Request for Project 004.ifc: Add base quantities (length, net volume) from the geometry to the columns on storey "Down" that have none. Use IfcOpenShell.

First a look at what the model holds.

```python
import ifcopenshell
import ifcopenshell.util.element
import ifcopenshell.util.unit

model = ifcopenshell.open("Project 004.ifc")
print(model.schema)
for unit_type in ("LENGTHUNIT", "AREAUNIT", "VOLUMEUNIT"):
    print(unit_type, ifcopenshell.util.unit.calculate_unit_scale(model, unit_type))
storey = next(s for s in model.by_type("IfcBuildingStorey") if s.Name == "Down")
columns = [e for e in ifcopenshell.util.element.get_decomposition(storey) if e.is_a("IfcColumn")]
for e in sorted(columns, key=lambda e: e.id()):
    print(e.id(), e.is_a(), e.Name, list(ifcopenshell.util.element.get_psets(e, qtos_only=True)), sep=" | ")
```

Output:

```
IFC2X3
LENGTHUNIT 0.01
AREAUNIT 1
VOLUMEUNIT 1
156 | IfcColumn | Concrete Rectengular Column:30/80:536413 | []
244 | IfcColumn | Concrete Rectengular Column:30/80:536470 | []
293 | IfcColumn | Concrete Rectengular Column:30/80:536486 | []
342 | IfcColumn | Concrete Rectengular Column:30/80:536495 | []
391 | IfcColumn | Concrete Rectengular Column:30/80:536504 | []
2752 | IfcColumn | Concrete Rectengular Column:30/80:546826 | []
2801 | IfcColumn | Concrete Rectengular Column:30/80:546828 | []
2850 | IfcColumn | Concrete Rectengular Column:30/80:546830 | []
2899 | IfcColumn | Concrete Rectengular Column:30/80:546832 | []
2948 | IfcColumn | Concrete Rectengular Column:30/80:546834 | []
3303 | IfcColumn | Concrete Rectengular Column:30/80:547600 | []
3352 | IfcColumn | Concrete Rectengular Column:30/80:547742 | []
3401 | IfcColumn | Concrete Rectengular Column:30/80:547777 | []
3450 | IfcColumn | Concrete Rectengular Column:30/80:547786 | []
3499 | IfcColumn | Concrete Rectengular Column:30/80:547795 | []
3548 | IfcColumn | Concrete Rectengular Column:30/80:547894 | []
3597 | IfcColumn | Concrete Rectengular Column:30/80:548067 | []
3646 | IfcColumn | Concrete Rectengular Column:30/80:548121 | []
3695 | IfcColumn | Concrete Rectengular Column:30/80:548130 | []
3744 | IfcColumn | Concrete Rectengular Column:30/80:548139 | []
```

```python
import ifcopenshell
import ifcopenshell.api.pset
import ifcopenshell.geom
import ifcopenshell.util.element
import ifcopenshell.util.shape
import ifcopenshell.util.unit

model = ifcopenshell.open("Project 004.ifc")
unit_scale = ifcopenshell.util.unit.calculate_unit_scale(model)
volume_scale = ifcopenshell.util.unit.calculate_unit_scale(model, "VOLUMEUNIT")
settings = ifcopenshell.geom.settings()

storey = next(s for s in model.by_type("IfcBuildingStorey") if s.Name == "Down")
columns = [e for e in ifcopenshell.util.element.get_decomposition(storey) if e.is_a("IfcColumn")]

for e in sorted(columns, key=lambda e: e.id()):
    if ifcopenshell.util.element.get_psets(e, qtos_only=True, should_inherit=False):
        continue
    # Geometry comes back in metres, in the element's own axes.
    shape = ifcopenshell.geom.create_shape(settings, e)
    values = {
        "Length": ifcopenshell.util.shape.get_z(shape.geometry) / unit_scale,
        "NetVolume": ifcopenshell.util.shape.get_volume(shape.geometry) / volume_scale,
    }
    qto = ifcopenshell.api.pset.add_qto(model, product=e, name="BaseQuantities")
    ifcopenshell.api.pset.edit_qto(model, qto=qto, properties=values)
    print(e.id(), {k: round(v, 3) for k, v in values.items()})

model.write("Project 004-out.ifc")
```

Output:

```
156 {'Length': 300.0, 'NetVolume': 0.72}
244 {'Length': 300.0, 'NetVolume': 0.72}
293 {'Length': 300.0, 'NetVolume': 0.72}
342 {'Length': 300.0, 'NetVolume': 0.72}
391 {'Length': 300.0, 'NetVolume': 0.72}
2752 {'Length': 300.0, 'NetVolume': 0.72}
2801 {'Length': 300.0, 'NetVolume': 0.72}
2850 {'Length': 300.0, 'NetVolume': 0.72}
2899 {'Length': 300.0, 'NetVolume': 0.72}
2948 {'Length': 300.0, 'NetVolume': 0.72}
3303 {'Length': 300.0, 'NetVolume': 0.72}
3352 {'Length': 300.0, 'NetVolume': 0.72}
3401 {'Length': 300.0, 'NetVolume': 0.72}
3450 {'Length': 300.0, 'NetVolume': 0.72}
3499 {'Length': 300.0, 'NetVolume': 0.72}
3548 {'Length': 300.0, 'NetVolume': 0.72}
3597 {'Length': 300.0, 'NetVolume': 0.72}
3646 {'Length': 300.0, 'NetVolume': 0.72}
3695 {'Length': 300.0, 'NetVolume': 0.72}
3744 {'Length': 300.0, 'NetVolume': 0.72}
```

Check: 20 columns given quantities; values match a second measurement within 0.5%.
